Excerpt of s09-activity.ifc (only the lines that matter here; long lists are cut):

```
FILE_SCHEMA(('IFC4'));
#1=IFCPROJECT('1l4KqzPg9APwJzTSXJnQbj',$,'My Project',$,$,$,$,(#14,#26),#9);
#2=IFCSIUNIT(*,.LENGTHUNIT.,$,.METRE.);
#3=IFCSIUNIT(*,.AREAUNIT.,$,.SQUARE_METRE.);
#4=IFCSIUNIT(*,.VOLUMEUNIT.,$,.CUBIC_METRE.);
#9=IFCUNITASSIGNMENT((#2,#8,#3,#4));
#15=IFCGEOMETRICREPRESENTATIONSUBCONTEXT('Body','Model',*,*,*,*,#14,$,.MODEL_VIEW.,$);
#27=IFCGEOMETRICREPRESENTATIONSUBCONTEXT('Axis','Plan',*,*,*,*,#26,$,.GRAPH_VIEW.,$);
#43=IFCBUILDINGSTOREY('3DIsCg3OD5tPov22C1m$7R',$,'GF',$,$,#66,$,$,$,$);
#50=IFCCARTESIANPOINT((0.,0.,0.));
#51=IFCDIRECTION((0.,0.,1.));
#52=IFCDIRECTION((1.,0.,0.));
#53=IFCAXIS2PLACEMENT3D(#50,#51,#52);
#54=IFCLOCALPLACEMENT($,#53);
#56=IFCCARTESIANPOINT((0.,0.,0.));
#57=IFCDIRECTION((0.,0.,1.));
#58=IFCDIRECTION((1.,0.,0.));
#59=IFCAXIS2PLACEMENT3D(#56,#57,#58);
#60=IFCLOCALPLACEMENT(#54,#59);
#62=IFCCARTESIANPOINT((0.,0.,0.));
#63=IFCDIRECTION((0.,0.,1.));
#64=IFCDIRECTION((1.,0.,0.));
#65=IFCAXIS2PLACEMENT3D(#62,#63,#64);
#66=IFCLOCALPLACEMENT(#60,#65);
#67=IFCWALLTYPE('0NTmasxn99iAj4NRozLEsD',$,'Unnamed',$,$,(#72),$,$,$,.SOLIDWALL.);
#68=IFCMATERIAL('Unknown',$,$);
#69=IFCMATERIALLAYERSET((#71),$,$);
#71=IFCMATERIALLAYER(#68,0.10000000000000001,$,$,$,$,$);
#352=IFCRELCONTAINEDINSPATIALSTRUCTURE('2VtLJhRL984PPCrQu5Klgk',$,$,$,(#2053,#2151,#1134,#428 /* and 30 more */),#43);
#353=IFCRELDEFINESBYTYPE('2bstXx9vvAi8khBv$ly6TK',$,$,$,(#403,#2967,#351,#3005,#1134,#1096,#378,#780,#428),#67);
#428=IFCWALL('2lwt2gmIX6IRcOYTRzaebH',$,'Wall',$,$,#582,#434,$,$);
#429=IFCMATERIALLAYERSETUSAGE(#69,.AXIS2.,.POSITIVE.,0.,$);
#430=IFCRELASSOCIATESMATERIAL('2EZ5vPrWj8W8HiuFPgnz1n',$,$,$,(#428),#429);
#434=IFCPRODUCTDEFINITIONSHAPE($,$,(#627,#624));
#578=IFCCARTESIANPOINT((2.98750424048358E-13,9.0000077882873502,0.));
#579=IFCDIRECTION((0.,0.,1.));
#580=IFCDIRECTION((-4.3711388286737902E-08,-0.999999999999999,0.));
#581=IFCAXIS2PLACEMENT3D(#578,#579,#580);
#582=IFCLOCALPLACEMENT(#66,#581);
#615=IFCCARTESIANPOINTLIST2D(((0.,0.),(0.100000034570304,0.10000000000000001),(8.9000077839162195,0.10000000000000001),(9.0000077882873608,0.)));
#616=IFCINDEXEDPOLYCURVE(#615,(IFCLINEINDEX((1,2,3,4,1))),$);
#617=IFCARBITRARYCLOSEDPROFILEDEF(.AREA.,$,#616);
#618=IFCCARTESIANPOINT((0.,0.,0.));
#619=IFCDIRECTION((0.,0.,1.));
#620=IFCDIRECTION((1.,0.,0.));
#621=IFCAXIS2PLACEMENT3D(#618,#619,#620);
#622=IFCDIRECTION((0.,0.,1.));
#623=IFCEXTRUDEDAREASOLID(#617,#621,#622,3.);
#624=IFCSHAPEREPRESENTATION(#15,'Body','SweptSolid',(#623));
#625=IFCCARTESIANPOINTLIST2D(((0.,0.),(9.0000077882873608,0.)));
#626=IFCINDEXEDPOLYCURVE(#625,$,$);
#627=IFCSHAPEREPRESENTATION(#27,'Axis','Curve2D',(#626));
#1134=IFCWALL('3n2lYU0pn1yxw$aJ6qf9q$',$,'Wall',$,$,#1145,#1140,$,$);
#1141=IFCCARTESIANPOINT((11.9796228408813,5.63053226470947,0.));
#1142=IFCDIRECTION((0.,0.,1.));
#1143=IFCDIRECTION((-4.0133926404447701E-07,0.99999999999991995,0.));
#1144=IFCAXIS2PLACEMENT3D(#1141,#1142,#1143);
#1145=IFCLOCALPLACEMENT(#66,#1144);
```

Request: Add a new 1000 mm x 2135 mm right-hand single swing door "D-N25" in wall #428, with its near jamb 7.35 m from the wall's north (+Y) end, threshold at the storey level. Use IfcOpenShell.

```python
import numpy as np
import ifcopenshell
import ifcopenshell.api.feature
import ifcopenshell.api.geometry
import ifcopenshell.api.root
import ifcopenshell.api.spatial
import ifcopenshell.geom
import ifcopenshell.util.element
import ifcopenshell.util.placement
import ifcopenshell.util.representation
import ifcopenshell.util.shape
import ifcopenshell.util.unit

model = ifcopenshell.open("s09-activity.ifc")
unit_scale = ifcopenshell.util.unit.calculate_unit_scale(model)
settings = ifcopenshell.geom.settings()


def volume(element):
    """Net volume in cubic metres, openings subtracted."""
    shape = ifcopenshell.geom.create_shape(settings, element)
    return ifcopenshell.util.shape.get_volume(shape.geometry)


wall = model.by_guid("2lwt2gmIX6IRcOYTRzaebH")
storey = ifcopenshell.util.element.get_container(wall, ifc_class="IfcBuildingStorey")
context = ifcopenshell.util.representation.get_context(model, "Model", "Body", "MODEL_VIEW")
before = volume(wall)

width, height, from_end, sill = 1, 2.135, 7.35, 0.0  # metres

# The wall runs along its own X axis, and the end named is its -X end.
wall_shape = ifcopenshell.geom.create_shape(settings, wall)
x, y, z = ifcopenshell.util.shape.get_vertices(wall_shape.geometry).T
start = x.min() + from_end
face, thickness = float(y.min()), float(y.max() - y.min())
wall_matrix = ifcopenshell.util.placement.get_local_placement(wall.ObjectPlacement)
level = ifcopenshell.util.placement.get_local_placement(storey.ObjectPlacement)[2, 3]


def in_wall(x, y):
    """Placement at x, y metres in the wall's axes, at sill height."""
    matrix = wall_matrix.copy()
    matrix[:, 3] = wall_matrix @ np.array([x / unit_scale, y / unit_scale, 0.0, 1.0])
    matrix[2, 3] = level + sill / unit_scale
    return matrix


# Opening: a box that overshoots both wall faces by 50 mm.
opening = ifcopenshell.api.root.create_entity(model, ifc_class="IfcOpeningElement", predefined_type="OPENING")
box = ifcopenshell.api.geometry.add_wall_representation(
    model, context=context, length=width, height=height, thickness=thickness + 0.1
)
ifcopenshell.api.geometry.assign_representation(model, product=opening, representation=box)
ifcopenshell.api.geometry.edit_object_placement(model, product=opening, matrix=in_wall(start, face - 0.05), is_si=False)
ifcopenshell.api.feature.add_feature(model, feature=opening, element=wall)

door = ifcopenshell.api.root.create_entity(model, ifc_class="IfcDoor", name="D-N25", predefined_type="DOOR")
door.OverallWidth, door.OverallHeight = width / unit_scale, height / unit_scale
door.OperationType = "SINGLE_SWING_RIGHT"
body = ifcopenshell.api.geometry.add_door_representation(
    model,
    context=context,
    overall_width=door.OverallWidth,
    overall_height=door.OverallHeight,
    operation_type="SINGLE_SWING_RIGHT",
    lining_properties={"LiningDepth": thickness / unit_scale, "ThresholdDepth": thickness / unit_scale},
)
ifcopenshell.api.geometry.assign_representation(model, product=door, representation=body)
ifcopenshell.api.spatial.assign_container(model, products=[door], relating_structure=storey)
ifcopenshell.api.feature.add_filling(model, opening=opening, element=door)

# The lining spans the wall, so the door starts at the wall face.
ifcopenshell.api.geometry.edit_object_placement(model, product=door, matrix=in_wall(start, face), is_si=False)

after = volume(wall)

print(f"wall volume {before:.3f} -> {after:.3f} m3")

model.write("s09-activity_edited.ifc")
```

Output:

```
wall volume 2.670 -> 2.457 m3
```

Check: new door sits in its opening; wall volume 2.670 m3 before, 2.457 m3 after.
